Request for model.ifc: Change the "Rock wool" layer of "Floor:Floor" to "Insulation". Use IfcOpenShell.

First a look at what the model holds.

```python
import ifcopenshell
import ifcopenshell.util.element

model = ifcopenshell.open("model.ifc")
print(model.schema)
for layer_set in model.by_type("IfcMaterialLayerSet"):
    if layer_set.LayerSetName == "Floor:Floor":
        for layer in layer_set.MaterialLayers:
            print(layer.id(), layer.Material and layer.Material.Name, layer.LayerThickness, sep=" | ")
        print(len(ifcopenshell.util.element.get_elements_by_material(model, layer_set)), "elements and types use it")
print(sorted(m.Name for m in model.by_type("IfcMaterial") if m.Name)[:60])
```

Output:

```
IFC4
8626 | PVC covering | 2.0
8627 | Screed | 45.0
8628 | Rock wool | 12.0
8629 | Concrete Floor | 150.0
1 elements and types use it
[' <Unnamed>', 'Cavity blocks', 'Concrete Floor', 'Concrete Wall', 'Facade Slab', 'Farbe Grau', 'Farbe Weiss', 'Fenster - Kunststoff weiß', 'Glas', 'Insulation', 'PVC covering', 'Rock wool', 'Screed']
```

```python
import ifcopenshell
import ifcopenshell.api.material

model = ifcopenshell.open("model.ifc")

layer_set = next(s for s in model.by_type("IfcMaterialLayerSet") if s.LayerSetName == "Floor:Floor")
layer = next(l for l in layer_set.MaterialLayers if l.Material and l.Material.Name == "Rock wool")
material = next(m for m in model.by_type("IfcMaterial") if m.Name == "Insulation")

# Point this one layer at the other material; renaming the old one would change it everywhere.
ifcopenshell.api.material.edit_layer(model, layer=layer, attributes={}, material=material)

print([l.Material.Name if l.Material else None for l in layer_set.MaterialLayers])

model.write("model_v2.ifc")
```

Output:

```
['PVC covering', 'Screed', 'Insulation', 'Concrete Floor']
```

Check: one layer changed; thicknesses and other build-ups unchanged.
